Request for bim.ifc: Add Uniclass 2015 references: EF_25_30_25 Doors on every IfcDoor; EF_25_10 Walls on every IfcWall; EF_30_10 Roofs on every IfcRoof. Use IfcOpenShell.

First a look at what the model holds.

```python
import ifcopenshell

model = ifcopenshell.open("bim.ifc")
print(model.schema)
print("classifications:", [c.Name for c in model.by_type("IfcClassification")])
for ifc_class in ("IfcDoor", "IfcRoof", "IfcStair", "IfcWall", "IfcWindow"):
    print(ifc_class, len(model.by_type(ifc_class)))
```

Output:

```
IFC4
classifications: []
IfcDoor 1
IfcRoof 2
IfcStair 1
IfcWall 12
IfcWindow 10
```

```python
import ifcopenshell
import ifcopenshell.api.classification

model = ifcopenshell.open("bim.ifc")

system = ifcopenshell.api.classification.add_classification(model, classification="Uniclass 2015")

codes = {
    "IfcDoor": ("EF_25_30_25", "Doors"),
    "IfcWall": ("EF_25_10", "Walls"),
    "IfcRoof": ("EF_30_10", "Roofs"),
}
for ifc_class, (code, name) in codes.items():
    products = model.by_type(ifc_class)
    ifcopenshell.api.classification.add_reference(
        model, products=products, classification=system, identification=code, name=name
    )
    print(code, len(products))

model.write("bim-out.ifc")
```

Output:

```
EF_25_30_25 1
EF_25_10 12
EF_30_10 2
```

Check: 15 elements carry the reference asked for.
